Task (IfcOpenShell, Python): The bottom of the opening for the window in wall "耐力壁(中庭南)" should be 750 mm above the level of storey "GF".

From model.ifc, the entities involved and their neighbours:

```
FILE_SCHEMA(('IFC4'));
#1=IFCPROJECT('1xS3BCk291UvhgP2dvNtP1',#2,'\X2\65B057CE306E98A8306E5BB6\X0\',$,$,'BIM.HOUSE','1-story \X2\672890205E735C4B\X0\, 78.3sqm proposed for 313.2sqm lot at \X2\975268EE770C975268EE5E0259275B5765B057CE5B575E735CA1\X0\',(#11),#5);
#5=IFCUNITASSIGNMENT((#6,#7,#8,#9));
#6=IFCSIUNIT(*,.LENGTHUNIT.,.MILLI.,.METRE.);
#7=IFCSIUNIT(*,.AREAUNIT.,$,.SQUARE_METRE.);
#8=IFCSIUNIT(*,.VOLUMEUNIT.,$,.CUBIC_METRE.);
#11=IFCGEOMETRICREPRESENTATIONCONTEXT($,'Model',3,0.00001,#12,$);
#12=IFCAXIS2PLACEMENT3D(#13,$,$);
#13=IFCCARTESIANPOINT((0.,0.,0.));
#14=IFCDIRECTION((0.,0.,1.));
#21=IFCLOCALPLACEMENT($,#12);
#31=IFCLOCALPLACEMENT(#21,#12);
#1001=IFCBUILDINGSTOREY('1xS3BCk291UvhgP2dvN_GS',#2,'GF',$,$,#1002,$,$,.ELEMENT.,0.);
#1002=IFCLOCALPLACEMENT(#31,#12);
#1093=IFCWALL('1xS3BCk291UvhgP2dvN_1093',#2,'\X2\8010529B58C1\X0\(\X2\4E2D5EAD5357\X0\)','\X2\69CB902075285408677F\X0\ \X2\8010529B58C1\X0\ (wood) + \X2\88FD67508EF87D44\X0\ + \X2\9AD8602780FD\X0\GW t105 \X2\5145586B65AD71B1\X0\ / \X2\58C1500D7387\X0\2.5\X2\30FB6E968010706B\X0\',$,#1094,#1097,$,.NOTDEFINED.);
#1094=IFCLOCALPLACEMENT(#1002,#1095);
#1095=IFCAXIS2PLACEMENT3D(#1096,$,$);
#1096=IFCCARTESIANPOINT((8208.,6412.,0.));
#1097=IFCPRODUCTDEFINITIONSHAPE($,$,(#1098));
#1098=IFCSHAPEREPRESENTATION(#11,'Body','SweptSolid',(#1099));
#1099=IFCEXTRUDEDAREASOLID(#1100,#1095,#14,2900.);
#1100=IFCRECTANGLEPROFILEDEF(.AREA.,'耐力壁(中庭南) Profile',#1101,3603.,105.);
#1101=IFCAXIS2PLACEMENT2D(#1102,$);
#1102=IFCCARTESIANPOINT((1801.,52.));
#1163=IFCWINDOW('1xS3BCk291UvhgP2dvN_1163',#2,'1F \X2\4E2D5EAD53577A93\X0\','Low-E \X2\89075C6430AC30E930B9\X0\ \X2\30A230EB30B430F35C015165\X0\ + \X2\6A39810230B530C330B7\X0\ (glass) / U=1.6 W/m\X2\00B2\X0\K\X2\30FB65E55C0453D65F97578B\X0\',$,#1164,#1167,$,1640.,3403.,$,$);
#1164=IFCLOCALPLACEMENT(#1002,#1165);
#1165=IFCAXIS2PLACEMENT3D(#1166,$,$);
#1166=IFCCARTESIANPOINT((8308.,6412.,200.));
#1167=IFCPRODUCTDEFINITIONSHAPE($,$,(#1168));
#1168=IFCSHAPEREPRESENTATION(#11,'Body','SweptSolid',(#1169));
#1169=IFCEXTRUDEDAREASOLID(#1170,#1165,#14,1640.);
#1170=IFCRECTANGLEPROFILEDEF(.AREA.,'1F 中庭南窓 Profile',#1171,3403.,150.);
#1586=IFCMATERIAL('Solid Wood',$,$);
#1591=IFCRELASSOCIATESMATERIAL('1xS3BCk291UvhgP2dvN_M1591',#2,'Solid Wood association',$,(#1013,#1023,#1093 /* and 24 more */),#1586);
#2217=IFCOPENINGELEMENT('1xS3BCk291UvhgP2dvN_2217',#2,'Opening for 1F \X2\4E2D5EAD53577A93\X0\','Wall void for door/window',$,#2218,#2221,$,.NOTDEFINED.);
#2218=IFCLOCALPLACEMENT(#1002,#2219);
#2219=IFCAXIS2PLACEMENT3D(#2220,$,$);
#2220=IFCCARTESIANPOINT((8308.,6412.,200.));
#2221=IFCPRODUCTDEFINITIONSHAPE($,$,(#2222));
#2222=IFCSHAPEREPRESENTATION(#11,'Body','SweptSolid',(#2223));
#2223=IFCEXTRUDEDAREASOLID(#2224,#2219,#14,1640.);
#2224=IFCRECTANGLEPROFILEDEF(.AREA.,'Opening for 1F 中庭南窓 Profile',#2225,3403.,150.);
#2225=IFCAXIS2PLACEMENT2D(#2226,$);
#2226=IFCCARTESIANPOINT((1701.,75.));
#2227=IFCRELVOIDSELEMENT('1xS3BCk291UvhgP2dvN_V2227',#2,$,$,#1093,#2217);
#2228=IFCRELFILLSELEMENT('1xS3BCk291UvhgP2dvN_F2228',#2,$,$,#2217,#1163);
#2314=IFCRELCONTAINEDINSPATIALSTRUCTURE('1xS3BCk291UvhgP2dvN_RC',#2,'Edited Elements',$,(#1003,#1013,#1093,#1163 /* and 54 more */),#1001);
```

```python
import numpy as np
import ifcopenshell
import ifcopenshell.api.geometry
import ifcopenshell.geom
import ifcopenshell.util.element
import ifcopenshell.util.placement
import ifcopenshell.util.shape
import ifcopenshell.util.unit

model = ifcopenshell.open("model.ifc")
unit_scale = ifcopenshell.util.unit.calculate_unit_scale(model)

window = model.by_guid("1xS3BCk291UvhgP2dvN_1163")
opening = window.FillsVoids[0].RelatingOpeningElement
storey = ifcopenshell.util.element.get_container(window, ifc_class="IfcBuildingStorey")
level = ifcopenshell.util.placement.get_local_placement(storey.ObjectPlacement)[2, 3]

# The opening's origin need not be at the sill, so measure its lowest point.
shape = ifcopenshell.geom.create_shape(ifcopenshell.geom.settings(), opening)
bottom = ifcopenshell.util.shape.get_shape_bottom_elevation(shape, shape.geometry) / unit_scale
dz = level + 0.75 / unit_scale - bottom

shift = np.array([0.0, 0.0, dz])
# The window is not placed relative to its opening, so move both.
for product in (opening, window):
    matrix = ifcopenshell.util.placement.get_local_placement(product.ObjectPlacement)
    matrix[:3, 3] += shift
    ifcopenshell.api.geometry.edit_object_placement(model, product=product, matrix=matrix, is_si=False)

print(f"moved by {dz * unit_scale:+.3f} m")

model.write("model-out.ifc")
```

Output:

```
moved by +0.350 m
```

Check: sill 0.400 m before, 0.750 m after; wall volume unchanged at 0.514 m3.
